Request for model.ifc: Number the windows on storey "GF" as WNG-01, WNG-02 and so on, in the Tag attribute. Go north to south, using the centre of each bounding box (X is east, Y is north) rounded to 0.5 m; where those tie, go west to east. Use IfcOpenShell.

First a look at what the model holds.

```python
import ifcopenshell
import ifcopenshell.util.element
import ifcopenshell.util.placement

model = ifcopenshell.open("model.ifc")
print(model.schema)
storey = next(s for s in model.by_type("IfcBuildingStorey") if s.Name == "GF")
windows = [e for e in ifcopenshell.util.element.get_decomposition(storey) if e.is_a("IfcWindow")]
for e in sorted(windows, key=lambda e: e.id()):
    origin = ifcopenshell.util.placement.get_local_placement(e.ObjectPlacement)[:3, 3]
    print(e.id(), e.Tag, e.Name, origin.round(2) + 0.0, sep=" | ")
```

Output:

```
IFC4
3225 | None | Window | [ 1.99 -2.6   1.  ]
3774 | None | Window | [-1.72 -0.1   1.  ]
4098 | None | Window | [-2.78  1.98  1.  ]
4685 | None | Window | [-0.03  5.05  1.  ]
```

```python
import ifcopenshell
import ifcopenshell.geom
import ifcopenshell.util.element
import ifcopenshell.util.shape

model = ifcopenshell.open("model.ifc")
settings = ifcopenshell.geom.settings()
settings.set("use-world-coords", True)


def centre(element):
    shape = ifcopenshell.geom.create_shape(settings, element)
    return ifcopenshell.util.shape.get_bbox_centroid(shape.geometry)


storey = next(s for s in model.by_type("IfcBuildingStorey") if s.Name == "GF")
windows = [e for e in ifcopenshell.util.element.get_decomposition(storey) if e.is_a("IfcWindow")]

# Insertion points can sit at a corner or the storey origin, so sort by the geometry (in metres).
centres = {e: centre(e) for e in windows}
windows.sort(key=lambda e: (-round(centres[e][1] / 0.5), centres[e][0]))

for i, e in enumerate(windows, start=1):
    number = f"WNG-{i:02d}"
    e.Tag = number
    print(e.id(), number)

model.write("model_edited.ifc")
```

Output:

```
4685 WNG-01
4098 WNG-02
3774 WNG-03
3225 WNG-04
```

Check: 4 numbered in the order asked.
